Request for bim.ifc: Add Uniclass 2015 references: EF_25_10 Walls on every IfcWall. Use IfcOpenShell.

First a look at what the model holds.

```python
import ifcopenshell

model = ifcopenshell.open("bim.ifc")
print(model.schema)
print("classifications:", [c.Name for c in model.by_type("IfcClassification")])
for ifc_class in ("IfcDoor", "IfcRoof", "IfcStair", "IfcWall", "IfcWindow"):
    print(ifc_class, len(model.by_type(ifc_class)))
```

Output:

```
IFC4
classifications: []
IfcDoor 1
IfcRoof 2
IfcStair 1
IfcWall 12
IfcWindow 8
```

```python
import ifcopenshell
import ifcopenshell.api.classification

model = ifcopenshell.open("bim.ifc")

system = ifcopenshell.api.classification.add_classification(model, classification="Uniclass 2015")

codes = {
    "IfcWall": ("EF_25_10", "Walls"),
}
for ifc_class, (code, name) in codes.items():
    products = model.by_type(ifc_class)
    ifcopenshell.api.classification.add_reference(
        model, products=products, classification=system, identification=code, name=name
    )
    print(code, len(products))

model.write("bim_v2.ifc")
```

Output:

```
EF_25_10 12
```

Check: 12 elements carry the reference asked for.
